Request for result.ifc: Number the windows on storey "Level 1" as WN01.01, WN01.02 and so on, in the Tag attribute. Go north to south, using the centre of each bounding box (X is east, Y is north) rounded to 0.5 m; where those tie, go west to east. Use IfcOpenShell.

First a look at what the model holds.

```python
import ifcopenshell
import ifcopenshell.util.element
import ifcopenshell.util.placement

model = ifcopenshell.open("result.ifc")
print(model.schema)
storey = next(s for s in model.by_type("IfcBuildingStorey") if s.Name == "Level 1")
windows = [e for e in ifcopenshell.util.element.get_decomposition(storey) if e.is_a("IfcWindow")]
for e in sorted(windows, key=lambda e: e.id()):
    origin = ifcopenshell.util.placement.get_local_placement(e.ObjectPlacement)[:3, 3]
    print(e.id(), e.Tag, e.Name, origin.round(2) + 0.0, sep=" | ")
```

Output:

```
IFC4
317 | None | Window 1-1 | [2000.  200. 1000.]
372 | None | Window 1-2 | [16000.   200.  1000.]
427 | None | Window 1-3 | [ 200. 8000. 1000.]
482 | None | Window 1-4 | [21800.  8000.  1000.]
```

```python
import ifcopenshell
import ifcopenshell.geom
import ifcopenshell.util.element
import ifcopenshell.util.shape

model = ifcopenshell.open("result.ifc")
settings = ifcopenshell.geom.settings()
settings.set("use-world-coords", True)


def centre(element):
    shape = ifcopenshell.geom.create_shape(settings, element)
    return ifcopenshell.util.shape.get_bbox_centroid(shape.geometry)


storey = next(s for s in model.by_type("IfcBuildingStorey") if s.Name == "Level 1")
windows = [e for e in ifcopenshell.util.element.get_decomposition(storey) if e.is_a("IfcWindow")]

# Insertion points can sit at a corner or the storey origin, so sort by the geometry (in metres).
centres = {e: centre(e) for e in windows}
windows.sort(key=lambda e: (-round(centres[e][1] / 0.5), centres[e][0]))

for i, e in enumerate(windows, start=1):
    number = f"WN01.{i:02d}"
    e.Tag = number
    print(e.id(), number)

model.write("result_edited.ifc")
```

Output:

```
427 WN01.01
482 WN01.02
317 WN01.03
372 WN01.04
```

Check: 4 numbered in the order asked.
